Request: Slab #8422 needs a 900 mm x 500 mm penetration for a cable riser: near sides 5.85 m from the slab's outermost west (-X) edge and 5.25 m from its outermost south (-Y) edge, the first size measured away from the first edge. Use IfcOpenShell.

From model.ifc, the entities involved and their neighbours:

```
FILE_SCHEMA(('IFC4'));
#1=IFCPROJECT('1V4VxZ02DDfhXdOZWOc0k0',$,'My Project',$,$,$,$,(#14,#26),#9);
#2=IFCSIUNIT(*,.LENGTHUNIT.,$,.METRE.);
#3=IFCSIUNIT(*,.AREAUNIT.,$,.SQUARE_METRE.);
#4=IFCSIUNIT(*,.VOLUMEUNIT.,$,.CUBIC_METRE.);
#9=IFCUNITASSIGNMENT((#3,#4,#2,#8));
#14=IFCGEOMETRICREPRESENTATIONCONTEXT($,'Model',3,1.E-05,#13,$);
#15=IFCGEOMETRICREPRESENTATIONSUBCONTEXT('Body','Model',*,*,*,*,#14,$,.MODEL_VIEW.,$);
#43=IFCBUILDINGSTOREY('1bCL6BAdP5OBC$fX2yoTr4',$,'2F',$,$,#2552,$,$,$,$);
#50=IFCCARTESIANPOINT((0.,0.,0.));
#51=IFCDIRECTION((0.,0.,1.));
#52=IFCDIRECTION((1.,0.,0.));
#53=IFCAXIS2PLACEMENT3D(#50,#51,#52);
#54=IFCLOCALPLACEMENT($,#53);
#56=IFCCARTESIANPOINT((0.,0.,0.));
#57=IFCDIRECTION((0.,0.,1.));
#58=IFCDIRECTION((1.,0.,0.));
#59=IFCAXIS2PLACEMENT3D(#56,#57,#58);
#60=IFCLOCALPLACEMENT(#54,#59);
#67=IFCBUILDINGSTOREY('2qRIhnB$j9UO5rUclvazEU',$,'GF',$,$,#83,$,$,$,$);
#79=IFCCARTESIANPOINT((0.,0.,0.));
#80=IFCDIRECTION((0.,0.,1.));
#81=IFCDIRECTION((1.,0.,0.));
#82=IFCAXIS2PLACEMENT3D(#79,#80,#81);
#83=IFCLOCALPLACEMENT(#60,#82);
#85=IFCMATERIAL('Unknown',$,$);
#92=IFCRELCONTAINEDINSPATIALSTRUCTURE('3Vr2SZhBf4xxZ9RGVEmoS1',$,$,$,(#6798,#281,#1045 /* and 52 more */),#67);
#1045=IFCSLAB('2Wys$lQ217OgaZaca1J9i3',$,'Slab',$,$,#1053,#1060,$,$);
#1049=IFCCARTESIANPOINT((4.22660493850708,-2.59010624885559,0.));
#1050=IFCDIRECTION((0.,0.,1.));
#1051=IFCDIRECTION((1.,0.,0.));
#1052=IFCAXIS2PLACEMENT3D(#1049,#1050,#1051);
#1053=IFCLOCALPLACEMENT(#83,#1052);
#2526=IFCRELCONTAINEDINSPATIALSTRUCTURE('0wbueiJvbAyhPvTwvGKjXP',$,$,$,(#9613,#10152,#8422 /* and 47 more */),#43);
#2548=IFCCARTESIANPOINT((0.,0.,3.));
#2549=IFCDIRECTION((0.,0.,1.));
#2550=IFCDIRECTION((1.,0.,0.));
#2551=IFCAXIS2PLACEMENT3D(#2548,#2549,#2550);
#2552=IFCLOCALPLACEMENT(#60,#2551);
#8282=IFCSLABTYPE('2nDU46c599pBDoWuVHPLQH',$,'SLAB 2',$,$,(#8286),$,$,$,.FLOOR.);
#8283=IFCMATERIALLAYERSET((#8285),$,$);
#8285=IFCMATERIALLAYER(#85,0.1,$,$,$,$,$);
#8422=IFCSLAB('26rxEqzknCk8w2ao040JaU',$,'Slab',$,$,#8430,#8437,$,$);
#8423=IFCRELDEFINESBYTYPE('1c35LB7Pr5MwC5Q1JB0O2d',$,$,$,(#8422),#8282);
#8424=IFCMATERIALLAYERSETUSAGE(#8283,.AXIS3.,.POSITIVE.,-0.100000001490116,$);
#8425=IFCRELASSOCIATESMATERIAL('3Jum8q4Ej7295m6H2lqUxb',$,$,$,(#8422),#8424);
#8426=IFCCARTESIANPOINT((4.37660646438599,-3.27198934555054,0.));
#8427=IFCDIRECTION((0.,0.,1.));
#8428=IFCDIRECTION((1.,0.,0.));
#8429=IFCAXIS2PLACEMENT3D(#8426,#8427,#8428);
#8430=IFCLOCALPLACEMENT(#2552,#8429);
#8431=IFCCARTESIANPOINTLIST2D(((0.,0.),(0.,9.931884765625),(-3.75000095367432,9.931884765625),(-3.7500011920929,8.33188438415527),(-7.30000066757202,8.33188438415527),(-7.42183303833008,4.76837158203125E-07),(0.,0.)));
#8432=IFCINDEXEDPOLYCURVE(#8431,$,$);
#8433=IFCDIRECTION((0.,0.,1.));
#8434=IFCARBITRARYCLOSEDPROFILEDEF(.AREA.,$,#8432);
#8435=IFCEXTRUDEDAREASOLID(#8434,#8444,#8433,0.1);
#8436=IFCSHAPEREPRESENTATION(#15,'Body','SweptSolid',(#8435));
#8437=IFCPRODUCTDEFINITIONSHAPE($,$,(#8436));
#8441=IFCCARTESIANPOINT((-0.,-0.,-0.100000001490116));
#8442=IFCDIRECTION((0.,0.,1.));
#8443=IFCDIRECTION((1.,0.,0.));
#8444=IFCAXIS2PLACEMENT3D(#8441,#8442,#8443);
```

```python
import numpy as np
import ifcopenshell
import ifcopenshell.api.feature
import ifcopenshell.api.geometry
import ifcopenshell.api.root
import ifcopenshell.geom
import ifcopenshell.util.placement
import ifcopenshell.util.representation
import ifcopenshell.util.shape
import ifcopenshell.util.unit

model = ifcopenshell.open("model.ifc")
unit_scale = ifcopenshell.util.unit.calculate_unit_scale(model)
settings = ifcopenshell.geom.settings()


def volume(element):
    """Net volume in cubic metres, openings subtracted."""
    shape = ifcopenshell.geom.create_shape(settings, element)
    return ifcopenshell.util.shape.get_volume(shape.geometry)


slab = model.by_id(8422)
before = volume(slab)

# Extent in the slab's own axes, in metres. The edges named are its -X and -Y sides.
slab_shape = ifcopenshell.geom.create_shape(settings, slab)
vertices = ifcopenshell.util.shape.get_vertices(slab_shape.geometry)
x_min, y_min, bottom = vertices.min(axis=0)
top = vertices[:, 2].max()

opening = ifcopenshell.api.root.create_entity(model, ifc_class="IfcOpeningElement", name="Cable riser opening", predefined_type="OPENING")
context = ifcopenshell.util.representation.get_context(model, "Model", "Body", "MODEL_VIEW")
width, depth = 0.9, 0.5
outline = [(0.0, 0.0), (width, 0.0), (width, depth), (0.0, depth), (0.0, 0.0)]
# Overshoot both faces by 50 mm so the cut is clean.
shape = ifcopenshell.api.geometry.add_slab_representation(
    model, context=context, depth=top - bottom + 0.1, polyline=outline
)
ifcopenshell.api.geometry.assign_representation(model, product=opening, representation=shape)

matrix = ifcopenshell.util.placement.get_local_placement(slab.ObjectPlacement)
matrix[:, 3] = matrix @ np.append(np.array([x_min + 5.85, y_min + 5.25, bottom - 0.05]) / unit_scale, 1.0)
ifcopenshell.api.geometry.edit_object_placement(model, product=opening, matrix=matrix, is_si=False)
ifcopenshell.api.feature.add_feature(model, feature=opening, element=slab)

after = volume(slab)

print(f"slab volume {before:.3f} -> {after:.3f} m3")

model.write("model_v2.ifc")
```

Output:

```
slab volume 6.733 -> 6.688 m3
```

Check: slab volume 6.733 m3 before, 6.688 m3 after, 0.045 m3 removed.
